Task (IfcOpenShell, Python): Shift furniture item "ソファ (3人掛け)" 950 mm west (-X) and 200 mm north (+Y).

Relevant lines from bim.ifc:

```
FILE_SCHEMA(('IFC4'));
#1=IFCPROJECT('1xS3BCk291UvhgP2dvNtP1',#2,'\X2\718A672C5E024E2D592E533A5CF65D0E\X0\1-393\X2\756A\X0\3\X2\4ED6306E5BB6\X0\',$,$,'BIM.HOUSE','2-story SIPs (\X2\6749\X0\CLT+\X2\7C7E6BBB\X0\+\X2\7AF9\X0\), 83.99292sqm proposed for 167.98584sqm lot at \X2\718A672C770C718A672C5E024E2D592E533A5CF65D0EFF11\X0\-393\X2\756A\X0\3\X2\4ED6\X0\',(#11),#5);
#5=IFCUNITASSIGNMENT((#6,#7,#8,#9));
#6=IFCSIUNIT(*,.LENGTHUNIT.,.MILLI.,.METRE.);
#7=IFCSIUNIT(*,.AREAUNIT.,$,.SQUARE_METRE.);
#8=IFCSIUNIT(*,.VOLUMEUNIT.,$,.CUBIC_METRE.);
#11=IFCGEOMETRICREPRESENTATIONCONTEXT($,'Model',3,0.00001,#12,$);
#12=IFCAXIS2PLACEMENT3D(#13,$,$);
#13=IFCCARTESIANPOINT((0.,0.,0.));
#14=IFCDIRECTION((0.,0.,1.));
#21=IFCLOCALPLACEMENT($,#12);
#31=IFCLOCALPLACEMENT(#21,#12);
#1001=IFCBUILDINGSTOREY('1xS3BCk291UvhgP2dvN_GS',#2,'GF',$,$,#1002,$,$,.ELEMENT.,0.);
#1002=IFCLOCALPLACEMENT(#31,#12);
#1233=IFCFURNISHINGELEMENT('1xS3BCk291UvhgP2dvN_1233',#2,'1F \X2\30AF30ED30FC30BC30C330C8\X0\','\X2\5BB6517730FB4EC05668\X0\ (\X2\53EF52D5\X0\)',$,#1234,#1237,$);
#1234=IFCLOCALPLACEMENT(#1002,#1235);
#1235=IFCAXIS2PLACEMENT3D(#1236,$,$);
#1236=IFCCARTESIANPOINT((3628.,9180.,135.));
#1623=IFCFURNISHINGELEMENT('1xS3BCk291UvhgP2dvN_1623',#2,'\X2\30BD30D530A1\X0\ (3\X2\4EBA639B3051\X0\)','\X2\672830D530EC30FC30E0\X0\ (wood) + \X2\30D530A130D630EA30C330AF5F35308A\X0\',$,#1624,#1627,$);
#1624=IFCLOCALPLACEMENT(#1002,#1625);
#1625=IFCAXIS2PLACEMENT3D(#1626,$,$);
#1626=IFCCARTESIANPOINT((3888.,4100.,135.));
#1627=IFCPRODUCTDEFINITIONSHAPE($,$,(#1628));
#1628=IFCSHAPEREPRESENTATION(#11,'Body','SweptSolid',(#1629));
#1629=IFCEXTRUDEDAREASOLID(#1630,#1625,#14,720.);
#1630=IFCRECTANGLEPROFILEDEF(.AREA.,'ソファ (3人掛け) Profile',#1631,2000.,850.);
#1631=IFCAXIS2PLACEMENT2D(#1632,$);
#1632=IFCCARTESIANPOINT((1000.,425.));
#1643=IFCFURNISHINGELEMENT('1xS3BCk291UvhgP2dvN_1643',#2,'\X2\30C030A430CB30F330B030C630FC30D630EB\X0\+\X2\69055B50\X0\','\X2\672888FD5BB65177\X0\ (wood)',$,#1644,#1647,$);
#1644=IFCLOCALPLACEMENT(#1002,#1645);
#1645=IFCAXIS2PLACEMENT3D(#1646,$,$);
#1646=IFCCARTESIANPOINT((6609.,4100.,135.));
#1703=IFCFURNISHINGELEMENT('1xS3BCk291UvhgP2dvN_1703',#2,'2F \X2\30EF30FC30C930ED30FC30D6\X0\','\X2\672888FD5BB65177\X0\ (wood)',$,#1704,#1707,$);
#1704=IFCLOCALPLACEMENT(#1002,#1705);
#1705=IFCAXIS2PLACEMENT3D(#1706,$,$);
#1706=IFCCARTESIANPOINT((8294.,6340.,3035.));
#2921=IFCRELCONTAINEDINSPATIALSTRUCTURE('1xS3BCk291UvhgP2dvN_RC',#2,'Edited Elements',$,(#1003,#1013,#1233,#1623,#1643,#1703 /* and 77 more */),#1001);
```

```python
import ifcopenshell
import ifcopenshell.api.geometry
import ifcopenshell.util.placement

model = ifcopenshell.open("bim.ifc")

item = model.by_guid("1xS3BCk291UvhgP2dvN_1623")
matrix = ifcopenshell.util.placement.get_local_placement(item.ObjectPlacement)
matrix[0, 3] -= 950.0
matrix[1, 3] += 200.0
ifcopenshell.api.geometry.edit_object_placement(model, product=item, matrix=matrix, is_si=False)

print(ifcopenshell.util.placement.get_local_placement(item.ObjectPlacement).round(3) + 0.0)

model.write("bim_rev.ifc")
```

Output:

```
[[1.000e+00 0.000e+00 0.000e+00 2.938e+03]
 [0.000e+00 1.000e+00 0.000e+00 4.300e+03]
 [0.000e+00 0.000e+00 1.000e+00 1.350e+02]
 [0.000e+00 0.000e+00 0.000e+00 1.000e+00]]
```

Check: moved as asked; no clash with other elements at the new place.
